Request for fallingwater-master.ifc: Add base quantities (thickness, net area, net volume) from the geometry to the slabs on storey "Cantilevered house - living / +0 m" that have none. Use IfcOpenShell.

First a look at what the model holds.

```python
import ifcopenshell
import ifcopenshell.util.element
import ifcopenshell.util.unit

model = ifcopenshell.open("fallingwater-master.ifc")
print(model.schema)
for unit_type in ("LENGTHUNIT", "AREAUNIT", "VOLUMEUNIT"):
    print(unit_type, ifcopenshell.util.unit.calculate_unit_scale(model, unit_type))
storey = next(s for s in model.by_type("IfcBuildingStorey") if s.Name == "Cantilevered house - living / +0 m")
slabs = [e for e in ifcopenshell.util.element.get_decomposition(storey) if e.is_a("IfcSlab")]
for e in sorted(slabs, key=lambda e: e.id()):
    print(e.id(), e.is_a(), e.Name, list(ifcopenshell.util.element.get_psets(e, qtos_only=True)), sep=" | ")
```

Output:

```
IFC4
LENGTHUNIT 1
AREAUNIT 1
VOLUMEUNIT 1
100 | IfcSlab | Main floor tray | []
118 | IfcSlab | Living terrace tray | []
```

```python
import ifcopenshell
import ifcopenshell.api.pset
import ifcopenshell.geom
import ifcopenshell.util.element
import ifcopenshell.util.shape
import ifcopenshell.util.unit

model = ifcopenshell.open("fallingwater-master.ifc")
unit_scale = ifcopenshell.util.unit.calculate_unit_scale(model)
area_scale = ifcopenshell.util.unit.calculate_unit_scale(model, "AREAUNIT")
volume_scale = ifcopenshell.util.unit.calculate_unit_scale(model, "VOLUMEUNIT")
settings = ifcopenshell.geom.settings()

storey = next(s for s in model.by_type("IfcBuildingStorey") if s.Name == "Cantilevered house - living / +0 m")
slabs = [e for e in ifcopenshell.util.element.get_decomposition(storey) if e.is_a("IfcSlab")]

for e in sorted(slabs, key=lambda e: e.id()):
    if ifcopenshell.util.element.get_psets(e, qtos_only=True, should_inherit=False):
        continue
    # Geometry comes back in metres, in the element's own axes.
    shape = ifcopenshell.geom.create_shape(settings, e)
    values = {
        "Width": ifcopenshell.util.shape.get_z(shape.geometry) / unit_scale,
        "NetArea": ifcopenshell.util.shape.get_footprint_area(shape.geometry) / area_scale,
        "NetVolume": ifcopenshell.util.shape.get_volume(shape.geometry) / volume_scale,
    }
    qto = ifcopenshell.api.pset.add_qto(model, product=e, name="Qto_SlabBaseQuantities")
    ifcopenshell.api.pset.edit_qto(model, qto=qto, properties=values)
    print(e.id(), {k: round(v, 3) for k, v in values.items()})

model.write("fallingwater-master_edited.ifc")
```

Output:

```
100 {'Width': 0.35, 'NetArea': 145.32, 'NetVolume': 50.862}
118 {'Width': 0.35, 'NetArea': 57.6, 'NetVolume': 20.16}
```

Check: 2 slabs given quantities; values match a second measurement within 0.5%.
